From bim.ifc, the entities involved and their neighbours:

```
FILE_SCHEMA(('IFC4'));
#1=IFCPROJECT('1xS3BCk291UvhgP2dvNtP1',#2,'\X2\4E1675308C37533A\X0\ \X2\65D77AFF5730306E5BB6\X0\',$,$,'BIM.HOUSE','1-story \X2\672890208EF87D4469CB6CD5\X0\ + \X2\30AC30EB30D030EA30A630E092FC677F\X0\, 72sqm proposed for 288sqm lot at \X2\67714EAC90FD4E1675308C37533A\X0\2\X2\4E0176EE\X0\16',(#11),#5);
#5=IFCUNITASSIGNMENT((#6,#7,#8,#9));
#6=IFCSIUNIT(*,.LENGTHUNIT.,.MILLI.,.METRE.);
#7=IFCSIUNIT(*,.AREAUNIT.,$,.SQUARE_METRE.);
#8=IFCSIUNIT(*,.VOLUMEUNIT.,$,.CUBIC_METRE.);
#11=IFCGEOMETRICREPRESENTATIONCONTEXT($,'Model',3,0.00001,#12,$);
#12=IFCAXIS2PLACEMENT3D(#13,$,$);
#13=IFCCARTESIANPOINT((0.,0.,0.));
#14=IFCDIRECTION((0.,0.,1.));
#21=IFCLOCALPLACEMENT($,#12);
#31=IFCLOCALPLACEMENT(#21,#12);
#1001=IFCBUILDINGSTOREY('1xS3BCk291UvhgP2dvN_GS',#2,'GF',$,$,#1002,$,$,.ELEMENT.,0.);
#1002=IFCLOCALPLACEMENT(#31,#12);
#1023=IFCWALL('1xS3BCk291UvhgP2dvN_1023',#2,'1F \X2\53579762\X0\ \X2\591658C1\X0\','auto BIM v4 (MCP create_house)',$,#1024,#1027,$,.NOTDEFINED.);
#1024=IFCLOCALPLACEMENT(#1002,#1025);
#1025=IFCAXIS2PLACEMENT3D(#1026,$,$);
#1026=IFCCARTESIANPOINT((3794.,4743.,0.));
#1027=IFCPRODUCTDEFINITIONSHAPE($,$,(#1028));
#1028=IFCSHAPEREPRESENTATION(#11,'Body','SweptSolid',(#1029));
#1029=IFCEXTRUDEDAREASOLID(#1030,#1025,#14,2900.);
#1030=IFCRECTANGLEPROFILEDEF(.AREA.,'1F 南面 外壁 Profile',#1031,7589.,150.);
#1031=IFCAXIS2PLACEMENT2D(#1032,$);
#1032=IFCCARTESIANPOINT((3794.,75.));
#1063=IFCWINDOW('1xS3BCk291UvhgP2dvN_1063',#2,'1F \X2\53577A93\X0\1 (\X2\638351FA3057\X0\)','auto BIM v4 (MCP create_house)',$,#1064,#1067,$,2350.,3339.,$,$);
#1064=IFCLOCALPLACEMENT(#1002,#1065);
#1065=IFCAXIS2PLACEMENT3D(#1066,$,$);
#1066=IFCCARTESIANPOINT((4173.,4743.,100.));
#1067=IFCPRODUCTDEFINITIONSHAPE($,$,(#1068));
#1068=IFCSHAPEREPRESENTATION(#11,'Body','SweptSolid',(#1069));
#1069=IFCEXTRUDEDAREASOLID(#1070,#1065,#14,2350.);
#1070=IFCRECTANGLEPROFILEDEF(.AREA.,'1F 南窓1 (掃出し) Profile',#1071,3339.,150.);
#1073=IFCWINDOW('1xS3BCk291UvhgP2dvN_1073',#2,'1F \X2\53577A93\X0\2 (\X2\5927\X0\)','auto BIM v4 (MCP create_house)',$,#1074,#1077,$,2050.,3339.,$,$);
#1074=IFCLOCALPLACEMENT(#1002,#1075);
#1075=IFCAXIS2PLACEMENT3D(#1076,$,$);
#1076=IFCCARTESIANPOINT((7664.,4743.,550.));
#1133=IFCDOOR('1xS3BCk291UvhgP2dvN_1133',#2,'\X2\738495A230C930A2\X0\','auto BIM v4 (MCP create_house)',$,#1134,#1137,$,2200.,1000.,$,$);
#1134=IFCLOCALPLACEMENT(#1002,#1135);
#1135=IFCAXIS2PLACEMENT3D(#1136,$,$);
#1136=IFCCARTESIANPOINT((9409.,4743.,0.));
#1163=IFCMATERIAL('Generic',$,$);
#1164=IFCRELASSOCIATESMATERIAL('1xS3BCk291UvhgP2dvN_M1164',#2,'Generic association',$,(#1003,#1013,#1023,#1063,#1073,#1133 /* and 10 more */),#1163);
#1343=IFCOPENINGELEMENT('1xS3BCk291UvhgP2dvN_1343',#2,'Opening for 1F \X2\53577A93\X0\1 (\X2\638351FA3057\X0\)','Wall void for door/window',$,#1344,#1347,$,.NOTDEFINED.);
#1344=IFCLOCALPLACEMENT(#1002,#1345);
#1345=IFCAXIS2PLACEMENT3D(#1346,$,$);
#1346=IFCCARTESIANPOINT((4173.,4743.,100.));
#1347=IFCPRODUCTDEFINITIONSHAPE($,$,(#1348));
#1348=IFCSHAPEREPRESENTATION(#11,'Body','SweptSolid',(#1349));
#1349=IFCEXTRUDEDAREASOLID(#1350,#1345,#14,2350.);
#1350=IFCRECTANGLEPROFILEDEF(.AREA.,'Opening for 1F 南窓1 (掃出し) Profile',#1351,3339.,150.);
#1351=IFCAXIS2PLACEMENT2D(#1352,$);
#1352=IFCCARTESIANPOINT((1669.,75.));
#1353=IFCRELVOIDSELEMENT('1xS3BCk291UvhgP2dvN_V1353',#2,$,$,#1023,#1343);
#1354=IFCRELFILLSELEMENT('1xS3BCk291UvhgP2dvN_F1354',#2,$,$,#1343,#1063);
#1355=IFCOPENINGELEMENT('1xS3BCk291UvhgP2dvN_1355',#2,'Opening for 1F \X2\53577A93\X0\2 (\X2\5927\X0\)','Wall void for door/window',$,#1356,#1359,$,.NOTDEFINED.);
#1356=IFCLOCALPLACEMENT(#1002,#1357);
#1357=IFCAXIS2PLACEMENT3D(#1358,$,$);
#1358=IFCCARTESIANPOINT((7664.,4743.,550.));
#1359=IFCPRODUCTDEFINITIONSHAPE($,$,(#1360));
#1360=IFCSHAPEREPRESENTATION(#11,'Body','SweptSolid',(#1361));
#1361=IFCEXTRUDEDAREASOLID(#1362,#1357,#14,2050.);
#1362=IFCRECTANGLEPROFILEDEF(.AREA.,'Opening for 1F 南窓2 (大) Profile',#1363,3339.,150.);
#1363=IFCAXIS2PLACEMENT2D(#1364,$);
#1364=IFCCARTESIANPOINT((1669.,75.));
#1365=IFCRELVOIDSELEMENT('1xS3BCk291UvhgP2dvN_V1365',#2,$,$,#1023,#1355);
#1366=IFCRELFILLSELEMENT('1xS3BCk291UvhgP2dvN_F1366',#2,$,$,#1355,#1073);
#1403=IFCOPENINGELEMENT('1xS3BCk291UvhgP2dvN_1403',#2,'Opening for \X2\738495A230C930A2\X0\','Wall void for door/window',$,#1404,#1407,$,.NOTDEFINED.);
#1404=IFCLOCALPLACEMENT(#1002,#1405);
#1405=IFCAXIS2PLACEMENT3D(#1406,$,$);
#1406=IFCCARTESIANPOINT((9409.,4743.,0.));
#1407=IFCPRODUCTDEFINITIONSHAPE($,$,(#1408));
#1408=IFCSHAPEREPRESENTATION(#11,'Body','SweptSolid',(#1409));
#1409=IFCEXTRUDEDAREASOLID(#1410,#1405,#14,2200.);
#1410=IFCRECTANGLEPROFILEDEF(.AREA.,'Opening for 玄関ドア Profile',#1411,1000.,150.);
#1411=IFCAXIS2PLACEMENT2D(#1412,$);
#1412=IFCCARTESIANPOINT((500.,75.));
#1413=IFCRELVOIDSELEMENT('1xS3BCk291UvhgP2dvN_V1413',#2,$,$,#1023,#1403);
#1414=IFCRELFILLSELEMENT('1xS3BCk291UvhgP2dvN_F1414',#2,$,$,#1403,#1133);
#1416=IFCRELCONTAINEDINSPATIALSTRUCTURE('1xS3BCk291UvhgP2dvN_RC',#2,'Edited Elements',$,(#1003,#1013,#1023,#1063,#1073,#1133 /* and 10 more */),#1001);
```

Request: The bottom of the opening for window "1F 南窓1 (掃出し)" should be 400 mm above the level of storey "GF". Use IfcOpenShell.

```python
import numpy as np
import ifcopenshell
import ifcopenshell.api.geometry
import ifcopenshell.geom
import ifcopenshell.util.element
import ifcopenshell.util.placement
import ifcopenshell.util.shape
import ifcopenshell.util.unit

model = ifcopenshell.open("bim.ifc")
unit_scale = ifcopenshell.util.unit.calculate_unit_scale(model)

window = model.by_guid("1xS3BCk291UvhgP2dvN_1063")
opening = window.FillsVoids[0].RelatingOpeningElement
storey = ifcopenshell.util.element.get_container(window, ifc_class="IfcBuildingStorey")
level = ifcopenshell.util.placement.get_local_placement(storey.ObjectPlacement)[2, 3]

# The opening's origin need not be at the sill, so measure its lowest point.
shape = ifcopenshell.geom.create_shape(ifcopenshell.geom.settings(), opening)
bottom = ifcopenshell.util.shape.get_shape_bottom_elevation(shape, shape.geometry) / unit_scale
dz = level + 0.4 / unit_scale - bottom

shift = np.array([0.0, 0.0, dz])
# The window is not placed relative to its opening, so move both.
for product in (opening, window):
    matrix = ifcopenshell.util.placement.get_local_placement(product.ObjectPlacement)
    matrix[:3, 3] += shift
    ifcopenshell.api.geometry.edit_object_placement(model, product=product, matrix=matrix, is_si=False)

print(f"moved by {dz * unit_scale:+.3f} m")

model.write("bim_rev.ifc")
```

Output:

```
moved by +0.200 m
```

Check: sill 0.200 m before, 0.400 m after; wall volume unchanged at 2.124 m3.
